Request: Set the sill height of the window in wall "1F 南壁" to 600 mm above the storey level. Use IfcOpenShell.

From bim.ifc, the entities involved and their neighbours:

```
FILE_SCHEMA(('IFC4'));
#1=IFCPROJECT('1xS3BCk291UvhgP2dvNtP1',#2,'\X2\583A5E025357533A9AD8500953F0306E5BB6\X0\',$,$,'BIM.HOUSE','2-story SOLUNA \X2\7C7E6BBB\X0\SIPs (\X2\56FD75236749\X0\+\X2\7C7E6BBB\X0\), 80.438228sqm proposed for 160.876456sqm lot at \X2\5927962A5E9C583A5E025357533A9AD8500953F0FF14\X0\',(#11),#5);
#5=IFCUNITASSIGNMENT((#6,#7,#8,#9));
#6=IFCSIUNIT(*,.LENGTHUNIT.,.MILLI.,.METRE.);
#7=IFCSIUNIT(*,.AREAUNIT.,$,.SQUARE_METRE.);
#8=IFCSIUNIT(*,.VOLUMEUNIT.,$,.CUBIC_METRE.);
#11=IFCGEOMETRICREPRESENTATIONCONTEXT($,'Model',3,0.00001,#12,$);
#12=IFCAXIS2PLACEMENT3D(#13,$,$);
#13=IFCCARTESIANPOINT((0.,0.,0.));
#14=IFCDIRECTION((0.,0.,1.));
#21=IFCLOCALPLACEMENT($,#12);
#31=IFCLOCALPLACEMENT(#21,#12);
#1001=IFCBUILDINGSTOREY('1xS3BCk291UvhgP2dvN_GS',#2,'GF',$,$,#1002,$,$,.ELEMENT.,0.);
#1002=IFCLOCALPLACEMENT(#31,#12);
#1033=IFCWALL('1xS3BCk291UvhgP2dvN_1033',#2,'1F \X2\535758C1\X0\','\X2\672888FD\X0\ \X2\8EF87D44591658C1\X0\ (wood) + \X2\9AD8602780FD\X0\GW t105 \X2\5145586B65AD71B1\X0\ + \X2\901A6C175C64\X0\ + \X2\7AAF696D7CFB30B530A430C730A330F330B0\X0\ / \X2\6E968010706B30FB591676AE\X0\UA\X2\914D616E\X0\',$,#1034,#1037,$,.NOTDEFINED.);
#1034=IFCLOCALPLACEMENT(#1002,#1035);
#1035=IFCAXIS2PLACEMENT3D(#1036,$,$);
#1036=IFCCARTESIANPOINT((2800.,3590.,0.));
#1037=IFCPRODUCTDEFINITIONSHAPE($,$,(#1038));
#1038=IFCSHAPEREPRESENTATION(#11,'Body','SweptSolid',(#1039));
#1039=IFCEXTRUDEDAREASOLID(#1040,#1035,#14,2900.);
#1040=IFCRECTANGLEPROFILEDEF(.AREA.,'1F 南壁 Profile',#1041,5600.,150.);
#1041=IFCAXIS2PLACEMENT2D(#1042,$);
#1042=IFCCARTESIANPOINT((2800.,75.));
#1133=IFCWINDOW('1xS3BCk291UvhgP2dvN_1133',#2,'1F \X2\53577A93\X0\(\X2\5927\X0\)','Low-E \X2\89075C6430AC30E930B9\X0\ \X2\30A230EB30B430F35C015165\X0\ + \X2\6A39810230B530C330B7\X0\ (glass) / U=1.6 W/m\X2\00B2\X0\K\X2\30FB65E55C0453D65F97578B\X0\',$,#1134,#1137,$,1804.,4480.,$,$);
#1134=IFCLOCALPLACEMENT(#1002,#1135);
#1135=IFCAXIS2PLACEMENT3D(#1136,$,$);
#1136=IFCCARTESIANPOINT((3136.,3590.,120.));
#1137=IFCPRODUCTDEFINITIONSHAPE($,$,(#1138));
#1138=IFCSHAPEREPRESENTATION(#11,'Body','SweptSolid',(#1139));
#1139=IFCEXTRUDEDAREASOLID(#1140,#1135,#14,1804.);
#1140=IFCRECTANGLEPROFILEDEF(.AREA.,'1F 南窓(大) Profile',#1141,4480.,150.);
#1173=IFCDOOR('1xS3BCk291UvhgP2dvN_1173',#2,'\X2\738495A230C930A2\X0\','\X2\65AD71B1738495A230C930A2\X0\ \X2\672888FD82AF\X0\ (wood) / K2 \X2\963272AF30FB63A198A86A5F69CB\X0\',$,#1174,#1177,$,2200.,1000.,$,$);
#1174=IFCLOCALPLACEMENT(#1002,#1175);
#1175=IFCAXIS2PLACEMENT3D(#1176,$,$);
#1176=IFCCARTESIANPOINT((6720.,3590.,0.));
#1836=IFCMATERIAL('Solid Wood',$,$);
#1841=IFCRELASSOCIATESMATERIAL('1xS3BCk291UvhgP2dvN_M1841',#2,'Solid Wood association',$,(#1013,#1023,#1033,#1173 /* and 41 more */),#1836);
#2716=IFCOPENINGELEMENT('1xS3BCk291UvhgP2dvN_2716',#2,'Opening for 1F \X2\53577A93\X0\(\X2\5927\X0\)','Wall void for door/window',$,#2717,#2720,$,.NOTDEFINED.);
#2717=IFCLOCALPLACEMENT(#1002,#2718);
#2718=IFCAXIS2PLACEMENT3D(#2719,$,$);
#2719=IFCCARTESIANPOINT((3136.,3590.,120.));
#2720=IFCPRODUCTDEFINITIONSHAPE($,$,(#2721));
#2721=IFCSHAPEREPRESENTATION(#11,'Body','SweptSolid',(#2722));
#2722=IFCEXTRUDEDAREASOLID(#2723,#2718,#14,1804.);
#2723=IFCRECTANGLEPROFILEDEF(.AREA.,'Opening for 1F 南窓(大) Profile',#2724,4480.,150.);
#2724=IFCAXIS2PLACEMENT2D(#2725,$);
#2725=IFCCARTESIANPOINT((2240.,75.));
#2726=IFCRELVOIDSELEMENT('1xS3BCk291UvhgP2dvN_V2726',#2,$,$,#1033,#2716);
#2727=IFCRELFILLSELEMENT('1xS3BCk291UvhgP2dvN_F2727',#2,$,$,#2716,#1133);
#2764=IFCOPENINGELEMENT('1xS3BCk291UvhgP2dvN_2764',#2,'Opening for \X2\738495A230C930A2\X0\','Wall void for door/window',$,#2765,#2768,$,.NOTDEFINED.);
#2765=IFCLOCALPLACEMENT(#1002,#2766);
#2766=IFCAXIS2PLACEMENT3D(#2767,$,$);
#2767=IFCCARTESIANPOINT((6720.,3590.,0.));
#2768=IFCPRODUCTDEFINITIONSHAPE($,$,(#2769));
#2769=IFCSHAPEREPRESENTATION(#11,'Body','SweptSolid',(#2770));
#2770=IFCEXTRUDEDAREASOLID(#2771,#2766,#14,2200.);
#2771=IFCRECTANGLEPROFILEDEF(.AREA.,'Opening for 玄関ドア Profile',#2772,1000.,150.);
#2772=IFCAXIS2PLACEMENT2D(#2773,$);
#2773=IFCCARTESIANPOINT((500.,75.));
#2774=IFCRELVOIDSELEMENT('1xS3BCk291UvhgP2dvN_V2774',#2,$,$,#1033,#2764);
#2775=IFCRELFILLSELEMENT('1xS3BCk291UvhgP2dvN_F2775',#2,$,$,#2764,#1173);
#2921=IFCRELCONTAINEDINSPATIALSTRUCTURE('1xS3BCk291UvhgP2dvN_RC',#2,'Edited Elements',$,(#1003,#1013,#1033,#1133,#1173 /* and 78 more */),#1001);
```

```python
import numpy as np
import ifcopenshell
import ifcopenshell.api.geometry
import ifcopenshell.geom
import ifcopenshell.util.element
import ifcopenshell.util.placement
import ifcopenshell.util.shape
import ifcopenshell.util.unit

model = ifcopenshell.open("bim.ifc")
unit_scale = ifcopenshell.util.unit.calculate_unit_scale(model)

window = model.by_guid("1xS3BCk291UvhgP2dvN_1133")
opening = window.FillsVoids[0].RelatingOpeningElement
storey = ifcopenshell.util.element.get_container(window, ifc_class="IfcBuildingStorey")
level = ifcopenshell.util.placement.get_local_placement(storey.ObjectPlacement)[2, 3]

# The opening's origin need not be at the sill, so measure its lowest point.
shape = ifcopenshell.geom.create_shape(ifcopenshell.geom.settings(), opening)
bottom = ifcopenshell.util.shape.get_shape_bottom_elevation(shape, shape.geometry) / unit_scale
dz = level + 0.6 / unit_scale - bottom

shift = np.array([0.0, 0.0, dz])
# The window is not placed relative to its opening, so move both.
for product in (opening, window):
    matrix = ifcopenshell.util.placement.get_local_placement(product.ObjectPlacement)
    matrix[:3, 3] += shift
    ifcopenshell.api.geometry.edit_object_placement(model, product=product, matrix=matrix, is_si=False)

print(f"moved by {dz * unit_scale:+.3f} m")

model.write("bim_rev.ifc")
```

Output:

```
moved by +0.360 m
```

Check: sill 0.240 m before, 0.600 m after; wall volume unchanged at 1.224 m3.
